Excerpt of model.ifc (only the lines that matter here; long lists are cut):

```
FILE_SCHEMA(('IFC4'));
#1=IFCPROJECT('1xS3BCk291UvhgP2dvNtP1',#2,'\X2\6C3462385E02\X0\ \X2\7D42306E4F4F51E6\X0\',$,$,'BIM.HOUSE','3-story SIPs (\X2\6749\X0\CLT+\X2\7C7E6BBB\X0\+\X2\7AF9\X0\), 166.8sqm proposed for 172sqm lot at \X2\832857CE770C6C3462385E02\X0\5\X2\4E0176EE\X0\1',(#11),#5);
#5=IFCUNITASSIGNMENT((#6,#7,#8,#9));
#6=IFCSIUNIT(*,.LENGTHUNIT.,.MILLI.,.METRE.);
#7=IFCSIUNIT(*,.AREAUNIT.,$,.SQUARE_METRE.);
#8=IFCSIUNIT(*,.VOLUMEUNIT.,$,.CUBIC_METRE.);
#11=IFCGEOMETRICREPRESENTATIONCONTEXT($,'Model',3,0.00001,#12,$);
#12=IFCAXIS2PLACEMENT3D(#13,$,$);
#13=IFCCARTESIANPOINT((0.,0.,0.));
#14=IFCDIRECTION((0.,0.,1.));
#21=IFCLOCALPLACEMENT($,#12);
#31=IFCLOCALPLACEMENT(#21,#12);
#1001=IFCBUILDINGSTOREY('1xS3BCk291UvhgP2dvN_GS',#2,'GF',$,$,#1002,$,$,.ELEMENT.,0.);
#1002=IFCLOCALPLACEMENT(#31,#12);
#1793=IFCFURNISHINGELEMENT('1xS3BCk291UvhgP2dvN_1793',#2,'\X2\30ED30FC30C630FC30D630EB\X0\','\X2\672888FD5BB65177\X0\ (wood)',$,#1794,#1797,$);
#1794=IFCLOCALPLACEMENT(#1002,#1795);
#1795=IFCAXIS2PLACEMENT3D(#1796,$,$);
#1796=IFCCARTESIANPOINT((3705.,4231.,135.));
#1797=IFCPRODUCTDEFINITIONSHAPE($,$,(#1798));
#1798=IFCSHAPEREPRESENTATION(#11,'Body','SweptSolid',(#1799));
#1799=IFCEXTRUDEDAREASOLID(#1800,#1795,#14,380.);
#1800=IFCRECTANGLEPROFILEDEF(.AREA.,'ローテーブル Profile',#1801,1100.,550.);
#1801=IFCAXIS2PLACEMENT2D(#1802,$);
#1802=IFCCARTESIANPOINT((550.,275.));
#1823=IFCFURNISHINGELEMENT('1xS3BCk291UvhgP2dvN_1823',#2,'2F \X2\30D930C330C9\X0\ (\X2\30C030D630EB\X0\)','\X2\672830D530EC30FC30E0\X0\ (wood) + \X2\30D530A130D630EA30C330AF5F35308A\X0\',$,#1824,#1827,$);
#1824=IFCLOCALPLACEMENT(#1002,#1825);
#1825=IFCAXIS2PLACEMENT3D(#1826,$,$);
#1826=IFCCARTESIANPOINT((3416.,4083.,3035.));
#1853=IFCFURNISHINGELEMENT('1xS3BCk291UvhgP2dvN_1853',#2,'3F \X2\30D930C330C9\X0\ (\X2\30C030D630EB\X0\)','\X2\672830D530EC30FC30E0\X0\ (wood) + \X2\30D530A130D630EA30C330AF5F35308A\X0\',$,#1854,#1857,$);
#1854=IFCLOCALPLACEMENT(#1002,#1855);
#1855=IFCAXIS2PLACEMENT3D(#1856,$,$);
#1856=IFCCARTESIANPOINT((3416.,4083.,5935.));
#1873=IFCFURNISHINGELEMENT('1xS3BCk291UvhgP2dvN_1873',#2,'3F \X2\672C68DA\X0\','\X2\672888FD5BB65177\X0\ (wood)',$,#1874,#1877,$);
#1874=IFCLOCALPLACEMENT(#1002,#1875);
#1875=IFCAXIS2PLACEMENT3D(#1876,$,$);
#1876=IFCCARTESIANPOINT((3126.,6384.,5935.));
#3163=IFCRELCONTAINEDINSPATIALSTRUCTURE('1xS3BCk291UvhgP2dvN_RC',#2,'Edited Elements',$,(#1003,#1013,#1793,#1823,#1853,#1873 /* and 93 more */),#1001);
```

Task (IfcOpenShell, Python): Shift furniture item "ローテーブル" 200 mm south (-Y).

```python
import ifcopenshell
import ifcopenshell.api.geometry
import ifcopenshell.util.placement
import ifcopenshell.util.unit

model = ifcopenshell.open("model.ifc")
unit_scale = ifcopenshell.util.unit.calculate_unit_scale(model)

item = model.by_guid("1xS3BCk291UvhgP2dvN_1793")
matrix = ifcopenshell.util.placement.get_local_placement(item.ObjectPlacement)
matrix[1, 3] -= 0.2 / unit_scale
ifcopenshell.api.geometry.edit_object_placement(model, product=item, matrix=matrix, is_si=False)

print(ifcopenshell.util.placement.get_local_placement(item.ObjectPlacement).round(3) + 0.0)

model.write("model_rev.ifc")
```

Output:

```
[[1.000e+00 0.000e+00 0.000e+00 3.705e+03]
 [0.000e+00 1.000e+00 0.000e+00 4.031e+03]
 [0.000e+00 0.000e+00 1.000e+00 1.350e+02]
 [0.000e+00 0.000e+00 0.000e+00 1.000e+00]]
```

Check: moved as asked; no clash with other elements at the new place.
